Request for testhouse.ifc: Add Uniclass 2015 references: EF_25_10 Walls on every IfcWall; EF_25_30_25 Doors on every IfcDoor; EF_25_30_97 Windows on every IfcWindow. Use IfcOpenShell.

First a look at what the model holds.

```python
import ifcopenshell

model = ifcopenshell.open("testhouse.ifc")
print(model.schema)
print("classifications:", [c.Name for c in model.by_type("IfcClassification")])
for ifc_class in ("IfcDoor", "IfcRoof", "IfcStair", "IfcWall", "IfcWindow"):
    print(ifc_class, len(model.by_type(ifc_class)))
```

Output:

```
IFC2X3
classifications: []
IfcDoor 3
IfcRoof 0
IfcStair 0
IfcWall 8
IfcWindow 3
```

```python
import ifcopenshell
import ifcopenshell.api.classification

model = ifcopenshell.open("testhouse.ifc")

# IFC2X3 requires Source and Edition and has no link from the project to the system.
system = model.create_entity("IfcClassification", Source="NBS", Edition="2015", Name="Uniclass 2015")

codes = {
    "IfcWall": ("EF_25_10", "Walls"),
    "IfcDoor": ("EF_25_30_25", "Doors"),
    "IfcWindow": ("EF_25_30_97", "Windows"),
}
for ifc_class, (code, name) in codes.items():
    products = model.by_type(ifc_class)
    ifcopenshell.api.classification.add_reference(
        model, products=products, classification=system, identification=code, name=name
    )
    print(code, len(products))

model.write("testhouse_edited.ifc")
```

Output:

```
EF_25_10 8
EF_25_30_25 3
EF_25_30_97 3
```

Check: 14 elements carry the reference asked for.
